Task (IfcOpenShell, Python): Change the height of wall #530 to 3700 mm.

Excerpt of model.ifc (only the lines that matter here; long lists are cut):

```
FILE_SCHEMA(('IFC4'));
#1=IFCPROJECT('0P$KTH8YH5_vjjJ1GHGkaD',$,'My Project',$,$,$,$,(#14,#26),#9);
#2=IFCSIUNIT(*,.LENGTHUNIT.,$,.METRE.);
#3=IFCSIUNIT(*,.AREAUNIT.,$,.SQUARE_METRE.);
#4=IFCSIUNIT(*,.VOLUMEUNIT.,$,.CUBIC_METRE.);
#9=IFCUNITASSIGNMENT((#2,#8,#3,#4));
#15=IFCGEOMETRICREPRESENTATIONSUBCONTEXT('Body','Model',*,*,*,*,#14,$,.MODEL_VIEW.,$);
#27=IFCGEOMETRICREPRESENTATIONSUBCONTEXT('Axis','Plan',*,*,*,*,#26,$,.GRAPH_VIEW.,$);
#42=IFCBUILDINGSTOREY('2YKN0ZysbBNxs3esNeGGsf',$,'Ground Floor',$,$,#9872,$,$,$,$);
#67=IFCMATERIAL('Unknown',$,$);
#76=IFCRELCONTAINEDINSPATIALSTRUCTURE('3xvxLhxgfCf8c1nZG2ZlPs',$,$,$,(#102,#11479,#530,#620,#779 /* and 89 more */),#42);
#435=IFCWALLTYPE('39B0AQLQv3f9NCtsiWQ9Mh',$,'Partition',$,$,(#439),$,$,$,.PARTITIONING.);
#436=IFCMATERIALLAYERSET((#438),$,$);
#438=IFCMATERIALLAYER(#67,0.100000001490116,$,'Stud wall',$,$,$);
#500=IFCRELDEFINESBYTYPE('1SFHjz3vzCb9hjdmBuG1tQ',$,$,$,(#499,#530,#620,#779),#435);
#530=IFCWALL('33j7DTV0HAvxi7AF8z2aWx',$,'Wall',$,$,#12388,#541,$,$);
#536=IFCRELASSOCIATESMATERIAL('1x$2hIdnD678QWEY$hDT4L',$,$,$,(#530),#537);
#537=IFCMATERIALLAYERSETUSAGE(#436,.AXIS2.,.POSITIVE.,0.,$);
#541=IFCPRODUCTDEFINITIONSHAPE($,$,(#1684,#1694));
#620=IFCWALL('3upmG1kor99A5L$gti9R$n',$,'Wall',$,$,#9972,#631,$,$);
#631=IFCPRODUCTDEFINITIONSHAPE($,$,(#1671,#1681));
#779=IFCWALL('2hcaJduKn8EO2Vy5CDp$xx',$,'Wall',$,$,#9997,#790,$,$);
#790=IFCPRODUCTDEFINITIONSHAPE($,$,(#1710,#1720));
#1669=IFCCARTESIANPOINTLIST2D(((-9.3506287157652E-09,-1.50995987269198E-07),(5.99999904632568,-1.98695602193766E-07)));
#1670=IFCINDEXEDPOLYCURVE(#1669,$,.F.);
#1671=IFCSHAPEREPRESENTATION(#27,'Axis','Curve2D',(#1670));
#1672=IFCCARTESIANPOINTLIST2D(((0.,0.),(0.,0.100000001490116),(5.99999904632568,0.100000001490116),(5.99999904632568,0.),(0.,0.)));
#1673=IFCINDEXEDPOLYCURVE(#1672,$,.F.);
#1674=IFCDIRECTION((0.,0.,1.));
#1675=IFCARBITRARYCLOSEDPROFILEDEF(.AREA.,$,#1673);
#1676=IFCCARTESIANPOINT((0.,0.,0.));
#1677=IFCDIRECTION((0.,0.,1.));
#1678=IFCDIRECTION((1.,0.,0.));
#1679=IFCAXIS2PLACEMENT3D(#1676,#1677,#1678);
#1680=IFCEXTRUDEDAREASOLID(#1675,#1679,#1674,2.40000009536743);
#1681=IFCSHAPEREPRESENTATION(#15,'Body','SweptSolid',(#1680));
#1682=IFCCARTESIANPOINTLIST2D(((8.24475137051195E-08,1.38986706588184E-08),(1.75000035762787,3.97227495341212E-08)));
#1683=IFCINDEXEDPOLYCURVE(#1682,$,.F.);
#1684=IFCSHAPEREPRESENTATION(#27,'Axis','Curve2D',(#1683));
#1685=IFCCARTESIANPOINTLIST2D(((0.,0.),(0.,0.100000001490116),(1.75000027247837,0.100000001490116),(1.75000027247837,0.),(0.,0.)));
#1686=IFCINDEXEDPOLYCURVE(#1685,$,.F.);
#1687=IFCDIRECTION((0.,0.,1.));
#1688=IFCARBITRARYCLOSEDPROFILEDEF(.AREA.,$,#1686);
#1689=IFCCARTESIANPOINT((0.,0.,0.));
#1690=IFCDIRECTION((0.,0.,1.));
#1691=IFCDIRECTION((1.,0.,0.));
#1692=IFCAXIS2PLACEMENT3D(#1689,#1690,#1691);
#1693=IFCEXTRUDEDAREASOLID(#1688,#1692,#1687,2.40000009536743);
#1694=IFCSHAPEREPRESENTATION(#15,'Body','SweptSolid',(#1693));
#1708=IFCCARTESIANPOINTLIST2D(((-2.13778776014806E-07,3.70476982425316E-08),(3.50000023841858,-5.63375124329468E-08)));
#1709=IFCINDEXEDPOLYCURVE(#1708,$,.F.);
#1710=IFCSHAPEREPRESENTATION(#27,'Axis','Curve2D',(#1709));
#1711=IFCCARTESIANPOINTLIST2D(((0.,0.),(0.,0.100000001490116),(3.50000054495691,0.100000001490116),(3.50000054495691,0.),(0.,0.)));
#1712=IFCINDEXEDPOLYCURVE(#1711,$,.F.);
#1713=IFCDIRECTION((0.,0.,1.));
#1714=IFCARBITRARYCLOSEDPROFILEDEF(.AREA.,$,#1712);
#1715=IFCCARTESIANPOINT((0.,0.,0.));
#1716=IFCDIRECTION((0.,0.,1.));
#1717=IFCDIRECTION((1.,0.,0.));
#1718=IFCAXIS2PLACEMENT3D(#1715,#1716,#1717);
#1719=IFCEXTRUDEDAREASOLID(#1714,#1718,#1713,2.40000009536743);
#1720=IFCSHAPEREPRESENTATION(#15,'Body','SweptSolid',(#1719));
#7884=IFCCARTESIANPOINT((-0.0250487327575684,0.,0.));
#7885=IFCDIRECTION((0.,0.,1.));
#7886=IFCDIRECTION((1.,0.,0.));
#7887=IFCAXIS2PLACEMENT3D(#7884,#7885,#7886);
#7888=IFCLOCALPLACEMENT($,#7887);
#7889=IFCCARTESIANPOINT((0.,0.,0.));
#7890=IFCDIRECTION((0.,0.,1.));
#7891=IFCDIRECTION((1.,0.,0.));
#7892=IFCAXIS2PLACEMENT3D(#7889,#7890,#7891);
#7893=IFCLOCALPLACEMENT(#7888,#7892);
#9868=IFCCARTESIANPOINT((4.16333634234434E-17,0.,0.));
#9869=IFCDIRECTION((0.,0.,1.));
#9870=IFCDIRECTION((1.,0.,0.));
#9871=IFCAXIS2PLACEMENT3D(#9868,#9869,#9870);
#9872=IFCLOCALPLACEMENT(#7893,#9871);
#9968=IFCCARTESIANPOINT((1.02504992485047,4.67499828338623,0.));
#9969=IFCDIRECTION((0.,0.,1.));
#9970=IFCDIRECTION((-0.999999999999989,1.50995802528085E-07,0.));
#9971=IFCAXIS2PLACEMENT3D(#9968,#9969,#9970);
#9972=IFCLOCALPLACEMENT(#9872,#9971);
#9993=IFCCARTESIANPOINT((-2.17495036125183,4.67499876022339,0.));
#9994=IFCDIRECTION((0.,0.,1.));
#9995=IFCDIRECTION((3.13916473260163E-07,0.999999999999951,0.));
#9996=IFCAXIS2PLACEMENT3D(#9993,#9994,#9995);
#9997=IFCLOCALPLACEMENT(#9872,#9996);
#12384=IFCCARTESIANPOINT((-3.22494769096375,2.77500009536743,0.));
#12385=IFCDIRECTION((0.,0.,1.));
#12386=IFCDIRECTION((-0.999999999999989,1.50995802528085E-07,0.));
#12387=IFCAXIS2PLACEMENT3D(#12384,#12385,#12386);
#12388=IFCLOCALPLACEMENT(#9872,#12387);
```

```python
import ifcopenshell
import ifcopenshell.geom
import ifcopenshell.util.representation
import ifcopenshell.util.shape
import ifcopenshell.util.unit

model = ifcopenshell.open("model.ifc")
unit_scale = ifcopenshell.util.unit.calculate_unit_scale(model)
settings = ifcopenshell.geom.settings()


def volume(element):
    """Net volume in cubic metres, openings subtracted."""
    shape = ifcopenshell.geom.create_shape(settings, element)
    return ifcopenshell.util.shape.get_volume(shape.geometry)


wall = model.by_guid("33j7DTV0HAvxi7AF8z2aWx")
before = volume(wall)

body = ifcopenshell.util.representation.get_representation(wall, "Model", "Body")
solid = body.Items[0]
old_height = solid.Depth
solid.Depth = 3.7 / unit_scale
after = volume(wall)

print(f"height {old_height:g} -> {solid.Depth:g}, volume {before:.3f} -> {after:.3f} m3")

model.write("model_edited.ifc")
```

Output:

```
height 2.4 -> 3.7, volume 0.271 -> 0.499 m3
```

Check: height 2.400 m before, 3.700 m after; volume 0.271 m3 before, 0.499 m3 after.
